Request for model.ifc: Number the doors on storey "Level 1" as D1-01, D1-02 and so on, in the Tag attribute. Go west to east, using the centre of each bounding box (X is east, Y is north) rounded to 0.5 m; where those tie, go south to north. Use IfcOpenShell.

First a look at what the model holds.

```python
import ifcopenshell
import ifcopenshell.util.element
import ifcopenshell.util.placement

model = ifcopenshell.open("model.ifc")
print(model.schema)
storey = next(s for s in model.by_type("IfcBuildingStorey") if s.Name == "Level 1")
doors = [e for e in ifcopenshell.util.element.get_decomposition(storey) if e.is_a("IfcDoor")]
for e in sorted(doors, key=lambda e: e.id()):
    origin = ifcopenshell.util.placement.get_local_placement(e.ObjectPlacement)[:3, 3]
    print(e.id(), e.Tag, e.Name, origin.round(2) + 0.0, sep=" | ")
```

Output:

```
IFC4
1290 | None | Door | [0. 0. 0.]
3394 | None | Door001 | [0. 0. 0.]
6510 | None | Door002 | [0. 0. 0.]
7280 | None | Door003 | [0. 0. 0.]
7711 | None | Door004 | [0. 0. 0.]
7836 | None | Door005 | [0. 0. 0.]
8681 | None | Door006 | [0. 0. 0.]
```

```python
import ifcopenshell
import ifcopenshell.geom
import ifcopenshell.util.element
import ifcopenshell.util.shape

model = ifcopenshell.open("model.ifc")
settings = ifcopenshell.geom.settings()
settings.set("use-world-coords", True)


def centre(element):
    shape = ifcopenshell.geom.create_shape(settings, element)
    return ifcopenshell.util.shape.get_bbox_centroid(shape.geometry)


storey = next(s for s in model.by_type("IfcBuildingStorey") if s.Name == "Level 1")
doors = [e for e in ifcopenshell.util.element.get_decomposition(storey) if e.is_a("IfcDoor")]

# Insertion points can sit at a corner or the storey origin, so sort by the geometry (in metres).
centres = {e: centre(e) for e in doors}
doors.sort(key=lambda e: (round(centres[e][0] / 0.5), centres[e][1]))

for i, e in enumerate(doors, start=1):
    number = f"D1-{i:02d}"
    e.Tag = number
    print(e.id(), number)

model.write("model_updated.ifc")
```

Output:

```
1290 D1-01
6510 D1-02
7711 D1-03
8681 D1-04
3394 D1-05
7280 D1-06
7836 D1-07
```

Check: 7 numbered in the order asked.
